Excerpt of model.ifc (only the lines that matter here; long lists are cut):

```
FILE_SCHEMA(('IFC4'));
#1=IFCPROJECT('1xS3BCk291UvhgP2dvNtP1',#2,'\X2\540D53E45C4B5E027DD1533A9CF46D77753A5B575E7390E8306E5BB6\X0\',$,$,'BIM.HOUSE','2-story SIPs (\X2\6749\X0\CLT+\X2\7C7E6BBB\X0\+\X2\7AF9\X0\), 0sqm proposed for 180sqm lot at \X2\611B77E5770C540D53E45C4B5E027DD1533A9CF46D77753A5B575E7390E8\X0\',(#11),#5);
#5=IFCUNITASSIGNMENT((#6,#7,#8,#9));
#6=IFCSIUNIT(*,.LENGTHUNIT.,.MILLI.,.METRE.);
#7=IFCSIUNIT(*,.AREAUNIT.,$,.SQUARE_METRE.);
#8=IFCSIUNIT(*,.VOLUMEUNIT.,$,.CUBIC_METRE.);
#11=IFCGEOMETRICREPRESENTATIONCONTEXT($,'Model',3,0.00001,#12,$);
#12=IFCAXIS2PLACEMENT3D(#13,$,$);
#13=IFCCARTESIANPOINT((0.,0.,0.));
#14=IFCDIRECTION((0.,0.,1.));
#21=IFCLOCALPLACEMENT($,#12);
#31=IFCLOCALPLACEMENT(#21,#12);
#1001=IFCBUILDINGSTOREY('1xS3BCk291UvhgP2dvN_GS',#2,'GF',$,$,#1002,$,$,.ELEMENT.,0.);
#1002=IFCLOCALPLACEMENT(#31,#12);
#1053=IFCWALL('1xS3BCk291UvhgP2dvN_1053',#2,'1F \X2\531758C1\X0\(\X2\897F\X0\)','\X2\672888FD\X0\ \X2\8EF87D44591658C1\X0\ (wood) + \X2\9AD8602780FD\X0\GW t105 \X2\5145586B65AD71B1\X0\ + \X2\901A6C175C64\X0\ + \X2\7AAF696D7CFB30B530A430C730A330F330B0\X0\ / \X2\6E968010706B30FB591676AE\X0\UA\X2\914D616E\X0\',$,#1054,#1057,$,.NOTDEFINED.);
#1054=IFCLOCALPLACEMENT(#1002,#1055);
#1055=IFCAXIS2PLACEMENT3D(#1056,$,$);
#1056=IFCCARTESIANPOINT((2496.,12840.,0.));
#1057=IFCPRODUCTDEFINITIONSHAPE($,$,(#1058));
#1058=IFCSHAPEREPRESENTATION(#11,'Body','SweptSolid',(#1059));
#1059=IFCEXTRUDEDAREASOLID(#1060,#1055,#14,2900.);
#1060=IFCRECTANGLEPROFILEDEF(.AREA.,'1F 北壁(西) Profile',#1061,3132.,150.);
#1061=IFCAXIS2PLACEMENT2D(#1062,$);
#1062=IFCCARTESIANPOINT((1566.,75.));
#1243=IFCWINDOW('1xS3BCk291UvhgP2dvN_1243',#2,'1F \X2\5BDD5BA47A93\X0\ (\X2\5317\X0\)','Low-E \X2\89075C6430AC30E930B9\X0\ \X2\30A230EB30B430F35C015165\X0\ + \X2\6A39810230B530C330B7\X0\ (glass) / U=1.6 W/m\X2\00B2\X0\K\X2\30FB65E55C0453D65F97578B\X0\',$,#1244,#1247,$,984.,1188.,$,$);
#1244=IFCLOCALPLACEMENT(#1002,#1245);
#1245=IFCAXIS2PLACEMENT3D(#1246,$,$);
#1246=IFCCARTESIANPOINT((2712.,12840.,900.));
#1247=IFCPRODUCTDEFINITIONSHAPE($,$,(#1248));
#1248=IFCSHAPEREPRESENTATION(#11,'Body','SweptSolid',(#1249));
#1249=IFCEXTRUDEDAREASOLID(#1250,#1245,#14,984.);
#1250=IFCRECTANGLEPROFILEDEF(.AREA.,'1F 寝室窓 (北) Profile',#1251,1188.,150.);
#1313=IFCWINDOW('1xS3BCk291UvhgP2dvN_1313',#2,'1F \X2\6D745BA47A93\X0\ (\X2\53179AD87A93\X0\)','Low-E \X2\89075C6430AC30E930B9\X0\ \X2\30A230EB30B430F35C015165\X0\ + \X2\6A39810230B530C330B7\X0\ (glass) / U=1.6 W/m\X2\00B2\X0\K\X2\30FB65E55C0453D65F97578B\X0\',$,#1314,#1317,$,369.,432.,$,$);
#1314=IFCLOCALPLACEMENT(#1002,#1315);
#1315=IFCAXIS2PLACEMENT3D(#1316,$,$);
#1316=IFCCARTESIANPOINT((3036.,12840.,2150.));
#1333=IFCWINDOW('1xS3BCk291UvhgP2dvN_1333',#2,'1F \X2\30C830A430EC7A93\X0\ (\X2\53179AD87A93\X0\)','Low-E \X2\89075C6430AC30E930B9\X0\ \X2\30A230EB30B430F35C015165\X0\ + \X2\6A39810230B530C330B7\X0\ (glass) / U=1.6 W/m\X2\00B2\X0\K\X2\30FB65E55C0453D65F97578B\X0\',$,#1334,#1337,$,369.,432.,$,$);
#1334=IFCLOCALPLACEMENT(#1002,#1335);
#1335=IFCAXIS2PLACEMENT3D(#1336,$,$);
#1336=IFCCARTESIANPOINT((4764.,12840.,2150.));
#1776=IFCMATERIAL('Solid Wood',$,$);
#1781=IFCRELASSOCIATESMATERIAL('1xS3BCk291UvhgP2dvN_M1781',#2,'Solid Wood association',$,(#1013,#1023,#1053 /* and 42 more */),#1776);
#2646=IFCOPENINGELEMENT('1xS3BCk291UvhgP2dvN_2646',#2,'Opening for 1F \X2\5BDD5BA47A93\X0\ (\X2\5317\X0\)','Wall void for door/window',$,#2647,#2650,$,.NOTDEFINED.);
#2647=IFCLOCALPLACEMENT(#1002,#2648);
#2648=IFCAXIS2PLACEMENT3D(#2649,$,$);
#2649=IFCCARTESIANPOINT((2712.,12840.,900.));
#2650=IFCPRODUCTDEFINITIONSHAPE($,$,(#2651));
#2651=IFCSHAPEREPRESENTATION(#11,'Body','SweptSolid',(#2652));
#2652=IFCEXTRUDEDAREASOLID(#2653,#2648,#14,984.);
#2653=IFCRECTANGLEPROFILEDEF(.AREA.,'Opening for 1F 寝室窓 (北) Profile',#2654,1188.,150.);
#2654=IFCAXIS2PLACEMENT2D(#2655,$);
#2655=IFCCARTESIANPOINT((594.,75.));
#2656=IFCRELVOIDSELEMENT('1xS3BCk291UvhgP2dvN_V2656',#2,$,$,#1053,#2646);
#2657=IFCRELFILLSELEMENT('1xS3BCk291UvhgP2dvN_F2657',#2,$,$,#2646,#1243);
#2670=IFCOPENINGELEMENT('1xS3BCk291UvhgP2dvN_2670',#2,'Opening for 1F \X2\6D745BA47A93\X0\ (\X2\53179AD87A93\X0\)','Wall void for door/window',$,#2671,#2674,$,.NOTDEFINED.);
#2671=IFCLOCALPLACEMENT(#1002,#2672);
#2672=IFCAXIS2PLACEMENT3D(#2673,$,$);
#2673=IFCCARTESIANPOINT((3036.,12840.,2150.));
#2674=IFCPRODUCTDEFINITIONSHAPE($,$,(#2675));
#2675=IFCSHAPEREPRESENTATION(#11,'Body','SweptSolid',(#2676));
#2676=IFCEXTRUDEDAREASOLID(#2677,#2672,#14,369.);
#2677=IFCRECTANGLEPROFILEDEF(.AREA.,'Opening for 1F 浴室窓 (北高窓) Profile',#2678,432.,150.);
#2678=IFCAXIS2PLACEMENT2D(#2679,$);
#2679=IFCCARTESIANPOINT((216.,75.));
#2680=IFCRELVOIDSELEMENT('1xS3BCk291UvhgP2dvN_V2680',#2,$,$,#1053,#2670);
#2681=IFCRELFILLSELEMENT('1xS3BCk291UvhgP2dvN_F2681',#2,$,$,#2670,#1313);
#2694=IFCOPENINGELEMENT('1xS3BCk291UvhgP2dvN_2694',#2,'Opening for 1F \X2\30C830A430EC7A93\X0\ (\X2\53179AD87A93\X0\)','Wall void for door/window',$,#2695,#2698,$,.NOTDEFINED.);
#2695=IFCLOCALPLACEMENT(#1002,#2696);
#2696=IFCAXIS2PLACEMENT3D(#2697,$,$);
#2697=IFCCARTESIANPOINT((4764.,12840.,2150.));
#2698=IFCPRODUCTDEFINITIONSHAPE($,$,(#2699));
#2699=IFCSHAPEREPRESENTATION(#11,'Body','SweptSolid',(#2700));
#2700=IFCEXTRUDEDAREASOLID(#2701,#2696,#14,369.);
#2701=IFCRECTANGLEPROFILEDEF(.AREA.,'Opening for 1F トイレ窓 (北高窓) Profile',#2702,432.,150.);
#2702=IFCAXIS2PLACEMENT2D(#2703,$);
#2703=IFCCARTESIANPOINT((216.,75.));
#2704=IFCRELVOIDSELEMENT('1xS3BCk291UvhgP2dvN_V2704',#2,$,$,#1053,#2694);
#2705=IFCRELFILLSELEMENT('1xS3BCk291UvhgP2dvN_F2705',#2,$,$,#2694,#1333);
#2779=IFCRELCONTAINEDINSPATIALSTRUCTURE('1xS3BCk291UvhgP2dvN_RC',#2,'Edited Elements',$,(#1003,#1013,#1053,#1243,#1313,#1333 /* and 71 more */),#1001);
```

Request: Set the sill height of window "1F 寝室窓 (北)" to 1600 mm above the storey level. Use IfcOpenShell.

```python
import numpy as np
import ifcopenshell
import ifcopenshell.api.geometry
import ifcopenshell.geom
import ifcopenshell.util.element
import ifcopenshell.util.placement
import ifcopenshell.util.shape
import ifcopenshell.util.unit

model = ifcopenshell.open("model.ifc")
unit_scale = ifcopenshell.util.unit.calculate_unit_scale(model)

window = model.by_guid("1xS3BCk291UvhgP2dvN_1243")
opening = window.FillsVoids[0].RelatingOpeningElement
storey = ifcopenshell.util.element.get_container(window, ifc_class="IfcBuildingStorey")
level = ifcopenshell.util.placement.get_local_placement(storey.ObjectPlacement)[2, 3]

# The opening's origin need not be at the sill, so measure its lowest point.
shape = ifcopenshell.geom.create_shape(ifcopenshell.geom.settings(), opening)
bottom = ifcopenshell.util.shape.get_shape_bottom_elevation(shape, shape.geometry) / unit_scale
dz = level + 1600.0 - bottom

shift = np.array([0.0, 0.0, dz])
# The window is not placed relative to its opening, so move both.
for product in (opening, window):
    matrix = ifcopenshell.util.placement.get_local_placement(product.ObjectPlacement)
    matrix[:3, 3] += shift
    ifcopenshell.api.geometry.edit_object_placement(model, product=product, matrix=matrix, is_si=False)

print(f"moved by {dz * unit_scale:+.3f} m")

model.write("model_edited.ifc")
```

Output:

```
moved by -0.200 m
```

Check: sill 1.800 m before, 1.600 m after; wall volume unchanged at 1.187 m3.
